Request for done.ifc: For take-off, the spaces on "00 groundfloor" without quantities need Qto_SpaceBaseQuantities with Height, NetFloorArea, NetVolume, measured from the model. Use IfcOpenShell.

First a look at what the model holds.

```python
import ifcopenshell
import ifcopenshell.util.element
import ifcopenshell.util.unit

model = ifcopenshell.open("done.ifc")
print(model.schema)
for unit_type in ("LENGTHUNIT", "AREAUNIT", "VOLUMEUNIT"):
    print(unit_type, ifcopenshell.util.unit.calculate_unit_scale(model, unit_type))
storey = next(s for s in model.by_type("IfcBuildingStorey") if s.Name == "00 groundfloor")
spaces = [e for e in ifcopenshell.util.element.get_decomposition(storey) if e.is_a("IfcSpace")]
for e in sorted(spaces, key=lambda e: e.id()):
    print(e.id(), e.is_a(), e.Name, list(ifcopenshell.util.element.get_psets(e, qtos_only=True)), sep=" | ")
```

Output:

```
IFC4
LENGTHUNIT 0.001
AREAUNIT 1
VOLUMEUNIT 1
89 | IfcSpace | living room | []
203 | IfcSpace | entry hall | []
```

```python
import ifcopenshell
import ifcopenshell.api.pset
import ifcopenshell.geom
import ifcopenshell.util.element
import ifcopenshell.util.shape
import ifcopenshell.util.unit

model = ifcopenshell.open("done.ifc")
unit_scale = ifcopenshell.util.unit.calculate_unit_scale(model)
area_scale = ifcopenshell.util.unit.calculate_unit_scale(model, "AREAUNIT")
volume_scale = ifcopenshell.util.unit.calculate_unit_scale(model, "VOLUMEUNIT")
settings = ifcopenshell.geom.settings()

storey = next(s for s in model.by_type("IfcBuildingStorey") if s.Name == "00 groundfloor")
spaces = [e for e in ifcopenshell.util.element.get_decomposition(storey) if e.is_a("IfcSpace")]

for e in sorted(spaces, key=lambda e: e.id()):
    if ifcopenshell.util.element.get_psets(e, qtos_only=True, should_inherit=False):
        continue
    # Geometry comes back in metres, in the element's own axes.
    shape = ifcopenshell.geom.create_shape(settings, e)
    values = {
        "Height": ifcopenshell.util.shape.get_z(shape.geometry) / unit_scale,
        "NetFloorArea": ifcopenshell.util.shape.get_footprint_area(shape.geometry) / area_scale,
        "NetVolume": ifcopenshell.util.shape.get_volume(shape.geometry) / volume_scale,
    }
    qto = ifcopenshell.api.pset.add_qto(model, product=e, name="Qto_SpaceBaseQuantities")
    ifcopenshell.api.pset.edit_qto(model, qto=qto, properties=values)
    print(e.id(), {k: round(v, 3) for k, v in values.items()})

model.write("done_edited.ifc")
```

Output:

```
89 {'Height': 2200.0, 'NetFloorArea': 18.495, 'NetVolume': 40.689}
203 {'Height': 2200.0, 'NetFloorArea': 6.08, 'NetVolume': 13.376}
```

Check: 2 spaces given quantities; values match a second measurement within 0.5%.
